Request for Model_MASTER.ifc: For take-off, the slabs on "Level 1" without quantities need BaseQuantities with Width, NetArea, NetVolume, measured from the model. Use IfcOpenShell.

First a look at what the model holds.

```python
import ifcopenshell
import ifcopenshell.util.element
import ifcopenshell.util.unit

model = ifcopenshell.open("Model_MASTER.ifc")
print(model.schema)
for unit_type in ("LENGTHUNIT", "AREAUNIT", "VOLUMEUNIT"):
    print(unit_type, ifcopenshell.util.unit.calculate_unit_scale(model, unit_type))
storey = next(s for s in model.by_type("IfcBuildingStorey") if s.Name == "Level 1")
slabs = [e for e in ifcopenshell.util.element.get_decomposition(storey) if e.is_a("IfcSlab")]
for e in sorted(slabs, key=lambda e: e.id()):
    print(e.id(), e.is_a(), e.Name, list(ifcopenshell.util.element.get_psets(e, qtos_only=True)), sep=" | ")
```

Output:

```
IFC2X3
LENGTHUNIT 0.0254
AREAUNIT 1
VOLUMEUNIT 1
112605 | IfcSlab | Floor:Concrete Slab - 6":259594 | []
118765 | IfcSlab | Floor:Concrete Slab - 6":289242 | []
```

```python
import ifcopenshell
import ifcopenshell.api.pset
import ifcopenshell.geom
import ifcopenshell.util.element
import ifcopenshell.util.shape
import ifcopenshell.util.unit

model = ifcopenshell.open("Model_MASTER.ifc")
unit_scale = ifcopenshell.util.unit.calculate_unit_scale(model)
area_scale = ifcopenshell.util.unit.calculate_unit_scale(model, "AREAUNIT")
volume_scale = ifcopenshell.util.unit.calculate_unit_scale(model, "VOLUMEUNIT")
settings = ifcopenshell.geom.settings()

storey = next(s for s in model.by_type("IfcBuildingStorey") if s.Name == "Level 1")
slabs = [e for e in ifcopenshell.util.element.get_decomposition(storey) if e.is_a("IfcSlab")]

for e in sorted(slabs, key=lambda e: e.id()):
    if ifcopenshell.util.element.get_psets(e, qtos_only=True, should_inherit=False):
        continue
    # Geometry comes back in metres, in the element's own axes.
    shape = ifcopenshell.geom.create_shape(settings, e)
    values = {
        "Width": ifcopenshell.util.shape.get_z(shape.geometry) / unit_scale,
        "NetArea": ifcopenshell.util.shape.get_footprint_area(shape.geometry) / area_scale,
        "NetVolume": ifcopenshell.util.shape.get_volume(shape.geometry) / volume_scale,
    }
    qto = ifcopenshell.api.pset.add_qto(model, product=e, name="BaseQuantities")
    ifcopenshell.api.pset.edit_qto(model, qto=qto, properties=values)
    print(e.id(), {k: round(v, 3) for k, v in values.items()})

model.write("Model_MASTER_updated.ifc")
```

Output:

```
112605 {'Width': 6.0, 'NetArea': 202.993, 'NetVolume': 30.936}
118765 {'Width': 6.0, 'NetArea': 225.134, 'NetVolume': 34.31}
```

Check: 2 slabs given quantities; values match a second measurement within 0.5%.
